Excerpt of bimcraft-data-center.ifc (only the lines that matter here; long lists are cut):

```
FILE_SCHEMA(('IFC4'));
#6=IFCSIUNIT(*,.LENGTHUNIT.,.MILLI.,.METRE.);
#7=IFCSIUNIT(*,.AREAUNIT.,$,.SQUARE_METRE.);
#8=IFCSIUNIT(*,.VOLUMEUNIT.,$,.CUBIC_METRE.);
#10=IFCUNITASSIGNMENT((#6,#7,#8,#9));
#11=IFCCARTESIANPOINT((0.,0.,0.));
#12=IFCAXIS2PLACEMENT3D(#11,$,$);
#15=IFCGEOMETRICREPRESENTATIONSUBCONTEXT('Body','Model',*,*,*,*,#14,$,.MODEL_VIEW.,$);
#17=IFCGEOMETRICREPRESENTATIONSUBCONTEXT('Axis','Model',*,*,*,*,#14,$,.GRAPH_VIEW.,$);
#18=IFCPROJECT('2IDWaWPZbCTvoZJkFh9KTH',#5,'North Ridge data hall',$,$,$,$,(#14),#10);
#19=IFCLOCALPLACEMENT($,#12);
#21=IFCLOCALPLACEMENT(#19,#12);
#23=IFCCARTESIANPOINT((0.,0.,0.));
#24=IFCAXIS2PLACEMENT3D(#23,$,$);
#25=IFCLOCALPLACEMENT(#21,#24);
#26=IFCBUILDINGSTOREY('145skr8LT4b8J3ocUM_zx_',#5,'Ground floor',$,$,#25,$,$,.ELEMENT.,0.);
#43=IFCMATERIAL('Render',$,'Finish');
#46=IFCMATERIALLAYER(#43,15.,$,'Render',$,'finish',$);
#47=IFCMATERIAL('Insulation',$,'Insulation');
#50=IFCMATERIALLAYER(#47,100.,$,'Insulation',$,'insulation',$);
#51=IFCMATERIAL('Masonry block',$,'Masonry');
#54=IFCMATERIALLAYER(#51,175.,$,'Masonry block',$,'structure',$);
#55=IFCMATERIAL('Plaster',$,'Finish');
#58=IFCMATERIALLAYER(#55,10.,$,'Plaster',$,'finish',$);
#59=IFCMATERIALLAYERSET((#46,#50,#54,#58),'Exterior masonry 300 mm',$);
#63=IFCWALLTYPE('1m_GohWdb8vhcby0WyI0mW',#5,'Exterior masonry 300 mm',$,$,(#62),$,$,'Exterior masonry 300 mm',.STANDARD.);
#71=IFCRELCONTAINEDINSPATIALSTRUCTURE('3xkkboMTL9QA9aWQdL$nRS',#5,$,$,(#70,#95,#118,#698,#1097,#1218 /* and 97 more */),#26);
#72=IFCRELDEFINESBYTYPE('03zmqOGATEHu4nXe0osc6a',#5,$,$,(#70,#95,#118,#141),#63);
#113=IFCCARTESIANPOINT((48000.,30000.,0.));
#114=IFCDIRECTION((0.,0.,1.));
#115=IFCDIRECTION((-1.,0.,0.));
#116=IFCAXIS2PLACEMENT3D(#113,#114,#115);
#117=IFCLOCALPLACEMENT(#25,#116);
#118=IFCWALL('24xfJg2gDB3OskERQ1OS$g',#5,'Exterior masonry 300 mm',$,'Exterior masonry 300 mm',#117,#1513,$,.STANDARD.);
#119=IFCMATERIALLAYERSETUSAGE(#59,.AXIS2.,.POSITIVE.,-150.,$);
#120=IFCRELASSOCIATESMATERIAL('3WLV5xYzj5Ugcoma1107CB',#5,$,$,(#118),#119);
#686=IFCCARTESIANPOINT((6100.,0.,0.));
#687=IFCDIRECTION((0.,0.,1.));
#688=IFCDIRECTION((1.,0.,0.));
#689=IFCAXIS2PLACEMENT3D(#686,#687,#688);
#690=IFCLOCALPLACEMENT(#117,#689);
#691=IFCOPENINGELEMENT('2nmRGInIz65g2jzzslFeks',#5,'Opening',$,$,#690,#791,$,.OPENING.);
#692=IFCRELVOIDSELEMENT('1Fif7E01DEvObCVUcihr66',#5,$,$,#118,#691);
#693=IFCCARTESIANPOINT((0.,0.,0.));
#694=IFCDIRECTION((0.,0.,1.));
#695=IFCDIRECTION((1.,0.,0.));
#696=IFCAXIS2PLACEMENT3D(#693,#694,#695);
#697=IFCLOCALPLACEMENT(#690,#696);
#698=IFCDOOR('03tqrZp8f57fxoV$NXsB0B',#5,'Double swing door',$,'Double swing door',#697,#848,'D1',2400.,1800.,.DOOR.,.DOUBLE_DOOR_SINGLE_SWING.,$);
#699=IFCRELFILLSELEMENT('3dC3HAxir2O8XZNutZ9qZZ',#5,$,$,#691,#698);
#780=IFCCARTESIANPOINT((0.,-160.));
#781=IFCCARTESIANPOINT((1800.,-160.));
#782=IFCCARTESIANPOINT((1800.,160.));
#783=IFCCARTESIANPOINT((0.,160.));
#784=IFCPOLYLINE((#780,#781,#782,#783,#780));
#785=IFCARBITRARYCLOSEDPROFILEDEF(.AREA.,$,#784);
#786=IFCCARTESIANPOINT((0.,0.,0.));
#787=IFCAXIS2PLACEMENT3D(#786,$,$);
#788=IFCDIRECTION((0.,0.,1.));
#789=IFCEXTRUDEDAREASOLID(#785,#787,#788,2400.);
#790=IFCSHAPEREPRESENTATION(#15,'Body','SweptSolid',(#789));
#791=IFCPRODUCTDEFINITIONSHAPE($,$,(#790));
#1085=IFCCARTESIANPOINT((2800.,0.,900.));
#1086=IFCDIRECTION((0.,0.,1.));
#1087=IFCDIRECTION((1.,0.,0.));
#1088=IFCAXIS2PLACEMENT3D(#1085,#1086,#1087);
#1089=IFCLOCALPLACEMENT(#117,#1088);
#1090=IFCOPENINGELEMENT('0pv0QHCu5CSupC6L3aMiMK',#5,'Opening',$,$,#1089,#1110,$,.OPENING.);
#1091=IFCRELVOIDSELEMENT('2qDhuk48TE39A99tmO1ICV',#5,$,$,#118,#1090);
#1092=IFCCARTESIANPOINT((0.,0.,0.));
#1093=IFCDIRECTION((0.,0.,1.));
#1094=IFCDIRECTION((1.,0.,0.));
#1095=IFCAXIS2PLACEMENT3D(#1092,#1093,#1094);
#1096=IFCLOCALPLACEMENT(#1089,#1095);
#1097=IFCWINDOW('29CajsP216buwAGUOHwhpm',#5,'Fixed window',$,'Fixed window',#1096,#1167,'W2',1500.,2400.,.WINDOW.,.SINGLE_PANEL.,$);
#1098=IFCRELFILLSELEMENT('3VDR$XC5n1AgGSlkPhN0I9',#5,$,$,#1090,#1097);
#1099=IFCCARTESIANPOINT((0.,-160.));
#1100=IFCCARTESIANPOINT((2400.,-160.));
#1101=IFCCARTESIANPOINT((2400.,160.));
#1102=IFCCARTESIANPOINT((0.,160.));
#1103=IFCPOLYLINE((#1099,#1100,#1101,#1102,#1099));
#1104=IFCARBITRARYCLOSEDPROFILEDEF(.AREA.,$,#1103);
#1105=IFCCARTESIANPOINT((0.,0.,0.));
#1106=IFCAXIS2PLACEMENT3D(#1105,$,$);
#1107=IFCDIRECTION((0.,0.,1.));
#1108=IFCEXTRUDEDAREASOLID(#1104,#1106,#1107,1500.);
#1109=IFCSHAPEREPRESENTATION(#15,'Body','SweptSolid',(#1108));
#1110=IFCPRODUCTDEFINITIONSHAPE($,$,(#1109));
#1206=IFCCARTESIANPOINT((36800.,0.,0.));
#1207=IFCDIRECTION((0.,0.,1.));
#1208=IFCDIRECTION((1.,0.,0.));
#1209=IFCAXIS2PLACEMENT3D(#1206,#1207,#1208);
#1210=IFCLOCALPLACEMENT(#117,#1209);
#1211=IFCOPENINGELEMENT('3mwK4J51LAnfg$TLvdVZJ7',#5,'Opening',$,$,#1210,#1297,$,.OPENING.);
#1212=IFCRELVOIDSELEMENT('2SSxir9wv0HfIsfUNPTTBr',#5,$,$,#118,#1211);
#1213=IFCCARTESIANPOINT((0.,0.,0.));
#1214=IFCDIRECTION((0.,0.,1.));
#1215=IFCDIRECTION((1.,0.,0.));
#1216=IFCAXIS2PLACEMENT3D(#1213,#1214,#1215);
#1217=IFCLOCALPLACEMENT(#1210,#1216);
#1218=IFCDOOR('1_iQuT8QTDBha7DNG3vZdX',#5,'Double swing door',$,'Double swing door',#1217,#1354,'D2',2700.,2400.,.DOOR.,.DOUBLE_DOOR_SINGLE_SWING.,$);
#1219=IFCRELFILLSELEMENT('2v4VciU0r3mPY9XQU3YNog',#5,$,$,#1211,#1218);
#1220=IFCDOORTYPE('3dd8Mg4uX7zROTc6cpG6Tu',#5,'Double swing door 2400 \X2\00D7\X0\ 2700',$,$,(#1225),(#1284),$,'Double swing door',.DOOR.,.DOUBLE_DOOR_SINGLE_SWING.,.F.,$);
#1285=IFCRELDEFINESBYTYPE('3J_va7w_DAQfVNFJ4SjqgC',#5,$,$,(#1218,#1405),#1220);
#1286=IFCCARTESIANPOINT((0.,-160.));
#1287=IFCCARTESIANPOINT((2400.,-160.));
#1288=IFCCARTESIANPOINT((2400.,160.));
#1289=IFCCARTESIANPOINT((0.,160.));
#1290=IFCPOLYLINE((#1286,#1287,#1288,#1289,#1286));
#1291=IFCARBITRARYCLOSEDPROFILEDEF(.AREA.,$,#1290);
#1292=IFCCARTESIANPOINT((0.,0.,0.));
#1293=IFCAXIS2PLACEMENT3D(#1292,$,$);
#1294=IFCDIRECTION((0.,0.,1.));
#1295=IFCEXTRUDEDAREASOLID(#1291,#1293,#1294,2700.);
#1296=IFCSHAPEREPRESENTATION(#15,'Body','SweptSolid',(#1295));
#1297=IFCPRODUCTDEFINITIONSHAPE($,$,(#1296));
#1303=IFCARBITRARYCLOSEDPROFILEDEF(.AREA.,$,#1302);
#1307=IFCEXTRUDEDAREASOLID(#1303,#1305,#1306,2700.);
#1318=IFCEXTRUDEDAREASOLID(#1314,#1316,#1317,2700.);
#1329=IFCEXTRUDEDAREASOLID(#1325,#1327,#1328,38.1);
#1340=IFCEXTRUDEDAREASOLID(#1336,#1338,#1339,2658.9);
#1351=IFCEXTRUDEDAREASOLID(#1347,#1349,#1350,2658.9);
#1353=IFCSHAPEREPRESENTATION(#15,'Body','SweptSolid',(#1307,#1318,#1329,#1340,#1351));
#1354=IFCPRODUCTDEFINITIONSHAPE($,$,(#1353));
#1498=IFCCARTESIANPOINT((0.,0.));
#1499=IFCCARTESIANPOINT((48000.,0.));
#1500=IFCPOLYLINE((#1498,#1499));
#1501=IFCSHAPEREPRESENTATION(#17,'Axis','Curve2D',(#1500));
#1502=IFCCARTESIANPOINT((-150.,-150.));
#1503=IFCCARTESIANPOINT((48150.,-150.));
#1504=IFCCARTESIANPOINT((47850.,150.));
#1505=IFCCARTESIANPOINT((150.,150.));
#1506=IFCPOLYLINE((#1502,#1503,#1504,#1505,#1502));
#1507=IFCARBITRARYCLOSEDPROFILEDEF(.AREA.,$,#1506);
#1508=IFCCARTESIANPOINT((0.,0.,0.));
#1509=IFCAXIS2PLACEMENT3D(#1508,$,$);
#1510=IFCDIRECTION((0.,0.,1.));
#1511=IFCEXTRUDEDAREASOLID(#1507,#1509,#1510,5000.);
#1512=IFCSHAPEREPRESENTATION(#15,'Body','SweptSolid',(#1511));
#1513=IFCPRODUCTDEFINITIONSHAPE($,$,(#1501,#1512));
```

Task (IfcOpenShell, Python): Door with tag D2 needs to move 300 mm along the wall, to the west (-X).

```python
import ifcopenshell
import ifcopenshell.api.geometry
import ifcopenshell.util.placement
import ifcopenshell.util.unit

model = ifcopenshell.open("bimcraft-data-center.ifc")
unit_scale = ifcopenshell.util.unit.calculate_unit_scale(model)

door = model.by_guid("1_iQuT8QTDBha7DNG3vZdX")
opening = door.FillsVoids[0].RelatingOpeningElement
wall = opening.VoidsElements[0].RelatingBuildingElement

wall_matrix = ifcopenshell.util.placement.get_local_placement(wall.ObjectPlacement)
shift = wall_matrix[:3, 0] * 0.3 / unit_scale
before = ifcopenshell.util.placement.get_local_placement(door.ObjectPlacement)[:3, 3].copy()

# The door is placed relative to its opening, so it follows when the opening moves.
matrix = ifcopenshell.util.placement.get_local_placement(opening.ObjectPlacement)
matrix[:3, 3] += shift
ifcopenshell.api.geometry.edit_object_placement(
    model, product=opening, matrix=matrix, is_si=False, should_transform_children=True
)

after = ifcopenshell.util.placement.get_local_placement(door.ObjectPlacement)[:3, 3]
print("door moved by", (after - before).round(3) + 0.0)

model.write("bimcraft-data-center_rev.ifc")
```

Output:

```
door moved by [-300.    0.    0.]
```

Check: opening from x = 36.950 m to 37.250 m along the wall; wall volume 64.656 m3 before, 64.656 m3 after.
